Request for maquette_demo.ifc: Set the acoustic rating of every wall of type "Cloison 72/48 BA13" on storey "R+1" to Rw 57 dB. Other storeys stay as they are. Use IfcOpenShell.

First a look at what the model holds.

```python
import ifcopenshell
import ifcopenshell.util.element

model = ifcopenshell.open("maquette_demo.ifc")
print(model.schema)
storey = next(s for s in model.by_type("IfcBuildingStorey") if s.Name == "R+1")
walls = [e for e in ifcopenshell.util.element.get_decomposition(storey) if e.is_a("IfcWall")]
seen = {}
for e in walls:
    element_type = ifcopenshell.util.element.get_type(e)
    key = (element_type.Name if element_type != e and element_type else None, ifcopenshell.util.element.get_pset(e, "Pset_WallCommon", "AcousticRating"))
    seen[key] = seen.get(key, 0) + 1
for (name, value), count in sorted(seen.items(), key=str):
    print(count, "x", name, "|", value)
```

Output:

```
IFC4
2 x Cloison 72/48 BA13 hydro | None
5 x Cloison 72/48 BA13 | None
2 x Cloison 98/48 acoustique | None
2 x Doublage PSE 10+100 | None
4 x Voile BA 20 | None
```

```python
import ifcopenshell
import ifcopenshell.api.pset
import ifcopenshell.util.element

model = ifcopenshell.open("maquette_demo.ifc")

storey = next(s for s in model.by_type("IfcBuildingStorey") if s.Name == "R+1")
walls = [e for e in ifcopenshell.util.element.get_decomposition(storey) if e.is_a("IfcWall")]

count = 0
for e in walls:
    element_type = ifcopenshell.util.element.get_type(e)
    if element_type in (None, e) or element_type.Name != "Cloison 72/48 BA13":
        continue
    # add_pset returns the element's existing set when there is one.
    pset = ifcopenshell.api.pset.add_pset(model, product=e, name="Pset_WallCommon")
    ifcopenshell.api.pset.edit_pset(model, pset=pset, properties={"AcousticRating": "Rw 57 dB"})
    count += 1

print(count, "walls updated")

model.write("maquette_demo_updated.ifc")
```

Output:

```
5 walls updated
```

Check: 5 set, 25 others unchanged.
